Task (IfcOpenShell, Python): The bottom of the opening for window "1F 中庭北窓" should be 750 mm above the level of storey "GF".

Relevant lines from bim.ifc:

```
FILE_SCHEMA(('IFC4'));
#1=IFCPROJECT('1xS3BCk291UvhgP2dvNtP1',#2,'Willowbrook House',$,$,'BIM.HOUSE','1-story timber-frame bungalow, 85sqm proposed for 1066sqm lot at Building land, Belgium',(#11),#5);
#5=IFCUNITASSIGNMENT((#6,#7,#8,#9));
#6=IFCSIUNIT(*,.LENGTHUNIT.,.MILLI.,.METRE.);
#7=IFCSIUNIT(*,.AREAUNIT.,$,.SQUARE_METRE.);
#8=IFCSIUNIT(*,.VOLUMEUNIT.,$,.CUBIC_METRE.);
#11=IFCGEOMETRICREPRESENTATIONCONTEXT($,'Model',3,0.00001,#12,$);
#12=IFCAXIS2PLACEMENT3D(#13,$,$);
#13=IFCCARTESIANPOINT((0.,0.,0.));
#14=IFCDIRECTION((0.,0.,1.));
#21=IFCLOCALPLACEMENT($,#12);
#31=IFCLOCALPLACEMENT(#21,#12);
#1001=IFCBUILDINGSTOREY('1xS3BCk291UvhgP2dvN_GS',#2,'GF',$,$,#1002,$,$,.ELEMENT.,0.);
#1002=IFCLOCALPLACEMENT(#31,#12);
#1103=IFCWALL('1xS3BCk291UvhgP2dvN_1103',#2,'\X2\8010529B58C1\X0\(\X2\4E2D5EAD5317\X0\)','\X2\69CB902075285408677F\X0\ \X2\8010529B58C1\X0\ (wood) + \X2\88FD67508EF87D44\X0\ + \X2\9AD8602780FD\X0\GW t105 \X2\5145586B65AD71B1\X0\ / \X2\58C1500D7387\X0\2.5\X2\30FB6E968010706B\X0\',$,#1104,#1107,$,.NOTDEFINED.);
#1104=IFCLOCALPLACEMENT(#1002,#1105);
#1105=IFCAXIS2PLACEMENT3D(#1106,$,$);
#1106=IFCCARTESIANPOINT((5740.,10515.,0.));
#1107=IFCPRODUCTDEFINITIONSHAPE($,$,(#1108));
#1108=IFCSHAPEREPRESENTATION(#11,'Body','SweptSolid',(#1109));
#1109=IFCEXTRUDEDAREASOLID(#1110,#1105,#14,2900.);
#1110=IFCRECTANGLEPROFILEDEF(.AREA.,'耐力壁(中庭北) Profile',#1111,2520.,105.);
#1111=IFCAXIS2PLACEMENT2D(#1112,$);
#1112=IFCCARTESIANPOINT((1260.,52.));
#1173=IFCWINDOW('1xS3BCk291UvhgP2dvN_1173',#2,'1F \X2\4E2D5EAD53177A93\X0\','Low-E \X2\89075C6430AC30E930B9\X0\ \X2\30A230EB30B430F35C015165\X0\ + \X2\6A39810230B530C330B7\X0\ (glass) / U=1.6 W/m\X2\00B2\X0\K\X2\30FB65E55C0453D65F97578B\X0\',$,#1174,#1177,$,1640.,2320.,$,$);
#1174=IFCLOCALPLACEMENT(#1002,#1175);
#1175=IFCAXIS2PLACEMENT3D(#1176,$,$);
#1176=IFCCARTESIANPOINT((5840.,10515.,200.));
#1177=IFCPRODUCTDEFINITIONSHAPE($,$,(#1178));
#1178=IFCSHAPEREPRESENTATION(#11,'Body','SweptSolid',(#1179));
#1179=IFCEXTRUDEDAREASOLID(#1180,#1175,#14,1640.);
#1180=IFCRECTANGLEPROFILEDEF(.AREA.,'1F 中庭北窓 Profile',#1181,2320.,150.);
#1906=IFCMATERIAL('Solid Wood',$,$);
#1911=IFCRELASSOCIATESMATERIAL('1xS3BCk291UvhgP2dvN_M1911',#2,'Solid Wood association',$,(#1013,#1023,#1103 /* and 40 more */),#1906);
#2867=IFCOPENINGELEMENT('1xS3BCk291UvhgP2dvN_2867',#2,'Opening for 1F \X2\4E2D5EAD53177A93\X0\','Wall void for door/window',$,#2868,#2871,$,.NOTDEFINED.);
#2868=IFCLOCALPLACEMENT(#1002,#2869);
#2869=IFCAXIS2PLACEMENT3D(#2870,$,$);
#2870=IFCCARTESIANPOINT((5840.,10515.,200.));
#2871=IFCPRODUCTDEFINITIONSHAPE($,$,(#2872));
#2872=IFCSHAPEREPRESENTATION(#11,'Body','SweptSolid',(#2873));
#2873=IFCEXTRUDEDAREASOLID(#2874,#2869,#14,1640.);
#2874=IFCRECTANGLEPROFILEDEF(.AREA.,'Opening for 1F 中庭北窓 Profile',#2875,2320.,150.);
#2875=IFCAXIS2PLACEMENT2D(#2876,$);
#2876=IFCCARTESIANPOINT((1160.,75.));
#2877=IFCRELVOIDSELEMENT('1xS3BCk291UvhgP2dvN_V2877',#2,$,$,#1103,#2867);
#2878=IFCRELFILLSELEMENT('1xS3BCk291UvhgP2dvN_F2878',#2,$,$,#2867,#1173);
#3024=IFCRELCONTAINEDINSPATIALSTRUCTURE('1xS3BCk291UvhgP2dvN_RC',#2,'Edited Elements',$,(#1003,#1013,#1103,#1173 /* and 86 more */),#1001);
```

```python
import numpy as np
import ifcopenshell
import ifcopenshell.api.geometry
import ifcopenshell.geom
import ifcopenshell.util.element
import ifcopenshell.util.placement
import ifcopenshell.util.shape
import ifcopenshell.util.unit

model = ifcopenshell.open("bim.ifc")
unit_scale = ifcopenshell.util.unit.calculate_unit_scale(model)

window = model.by_id(1173)
opening = window.FillsVoids[0].RelatingOpeningElement
storey = ifcopenshell.util.element.get_container(window, ifc_class="IfcBuildingStorey")
level = ifcopenshell.util.placement.get_local_placement(storey.ObjectPlacement)[2, 3]

# The opening's origin need not be at the sill, so measure its lowest point.
shape = ifcopenshell.geom.create_shape(ifcopenshell.geom.settings(), opening)
bottom = ifcopenshell.util.shape.get_shape_bottom_elevation(shape, shape.geometry) / unit_scale
dz = level + 0.75 / unit_scale - bottom

shift = np.array([0.0, 0.0, dz])
# The window is not placed relative to its opening, so move both.
for product in (opening, window):
    matrix = ifcopenshell.util.placement.get_local_placement(product.ObjectPlacement)
    matrix[:3, 3] += shift
    ifcopenshell.api.geometry.edit_object_placement(model, product=product, matrix=matrix, is_si=False)

print(f"moved by {dz * unit_scale:+.3f} m")

model.write("bim_updated.ifc")
```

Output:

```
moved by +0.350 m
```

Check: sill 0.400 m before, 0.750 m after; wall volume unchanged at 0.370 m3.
